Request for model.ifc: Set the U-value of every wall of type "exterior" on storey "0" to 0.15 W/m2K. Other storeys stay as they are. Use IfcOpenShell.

First a look at what the model holds.

```python
import ifcopenshell
import ifcopenshell.util.element

model = ifcopenshell.open("model.ifc")
print(model.schema)
storey = next(s for s in model.by_type("IfcBuildingStorey") if s.Name == "0")
walls = [e for e in ifcopenshell.util.element.get_decomposition(storey) if e.is_a("IfcWall")]
seen = {}
for e in walls:
    element_type = ifcopenshell.util.element.get_type(e)
    key = (element_type.Name if element_type != e and element_type else None, ifcopenshell.util.element.get_pset(e, "Pset_WallCommon", "ThermalTransmittance"))
    seen[key] = seen.get(key, 0) + 1
for (name, value), count in sorted(seen.items(), key=str):
    print(count, "x", name, "|", value)
```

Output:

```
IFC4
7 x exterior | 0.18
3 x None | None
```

```python
import ifcopenshell
import ifcopenshell.api.pset
import ifcopenshell.util.element

model = ifcopenshell.open("model.ifc")

storey = next(s for s in model.by_type("IfcBuildingStorey") if s.Name == "0")
walls = [e for e in ifcopenshell.util.element.get_decomposition(storey) if e.is_a("IfcWall")]

count = 0
for e in walls:
    element_type = ifcopenshell.util.element.get_type(e)
    if element_type in (None, e) or element_type.Name != "exterior":
        continue
    # add_pset returns the element's existing set when there is one.
    pset = ifcopenshell.api.pset.add_pset(model, product=e, name="Pset_WallCommon")
    ifcopenshell.api.pset.edit_pset(model, pset=pset, properties={"ThermalTransmittance": 0.15})
    count += 1

print(count, "walls updated")

model.write("model-out.ifc")
```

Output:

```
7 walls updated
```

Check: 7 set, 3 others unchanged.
